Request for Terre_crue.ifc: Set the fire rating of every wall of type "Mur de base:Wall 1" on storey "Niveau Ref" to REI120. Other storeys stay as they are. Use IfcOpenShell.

First a look at what the model holds.

```python
import ifcopenshell
import ifcopenshell.util.element

model = ifcopenshell.open("Terre_crue.ifc")
print(model.schema)
storey = next(s for s in model.by_type("IfcBuildingStorey") if s.Name == "Niveau Ref")
walls = [e for e in ifcopenshell.util.element.get_decomposition(storey) if e.is_a("IfcWall")]
seen = {}
for e in walls:
    element_type = ifcopenshell.util.element.get_type(e)
    key = (element_type.Name if element_type != e and element_type else None, ifcopenshell.util.element.get_pset(e, "Pset_WallCommon", "FireRating"))
    seen[key] = seen.get(key, 0) + 1
for (name, value), count in sorted(seen.items(), key=str):
    print(count, "x", name, "|", value)
```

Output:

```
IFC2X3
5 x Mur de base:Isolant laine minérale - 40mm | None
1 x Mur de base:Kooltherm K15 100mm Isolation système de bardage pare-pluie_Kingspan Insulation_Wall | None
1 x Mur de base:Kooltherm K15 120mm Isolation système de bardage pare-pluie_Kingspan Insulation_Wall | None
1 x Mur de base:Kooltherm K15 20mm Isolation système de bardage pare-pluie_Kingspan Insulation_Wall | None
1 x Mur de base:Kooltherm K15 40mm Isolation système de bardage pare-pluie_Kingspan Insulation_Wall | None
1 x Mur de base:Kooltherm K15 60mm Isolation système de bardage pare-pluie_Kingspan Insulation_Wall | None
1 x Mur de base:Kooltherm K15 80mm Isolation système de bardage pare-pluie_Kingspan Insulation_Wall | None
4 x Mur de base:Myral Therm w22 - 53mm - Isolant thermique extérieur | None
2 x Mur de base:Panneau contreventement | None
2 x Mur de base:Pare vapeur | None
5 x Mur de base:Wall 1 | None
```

```python
import ifcopenshell
import ifcopenshell.api.pset
import ifcopenshell.util.element

model = ifcopenshell.open("Terre_crue.ifc")

storey = next(s for s in model.by_type("IfcBuildingStorey") if s.Name == "Niveau Ref")
walls = [e for e in ifcopenshell.util.element.get_decomposition(storey) if e.is_a("IfcWall")]

count = 0
for e in walls:
    element_type = ifcopenshell.util.element.get_type(e)
    if element_type in (None, e) or element_type.Name != "Mur de base:Wall 1":
        continue
    # add_pset returns the element's existing set when there is one.
    pset = ifcopenshell.api.pset.add_pset(model, product=e, name="Pset_WallCommon")
    ifcopenshell.api.pset.edit_pset(model, pset=pset, properties={"FireRating": "REI120"})
    count += 1

print(count, "walls updated")

model.write("Terre_crue_rev.ifc")
```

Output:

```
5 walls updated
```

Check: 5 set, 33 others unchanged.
